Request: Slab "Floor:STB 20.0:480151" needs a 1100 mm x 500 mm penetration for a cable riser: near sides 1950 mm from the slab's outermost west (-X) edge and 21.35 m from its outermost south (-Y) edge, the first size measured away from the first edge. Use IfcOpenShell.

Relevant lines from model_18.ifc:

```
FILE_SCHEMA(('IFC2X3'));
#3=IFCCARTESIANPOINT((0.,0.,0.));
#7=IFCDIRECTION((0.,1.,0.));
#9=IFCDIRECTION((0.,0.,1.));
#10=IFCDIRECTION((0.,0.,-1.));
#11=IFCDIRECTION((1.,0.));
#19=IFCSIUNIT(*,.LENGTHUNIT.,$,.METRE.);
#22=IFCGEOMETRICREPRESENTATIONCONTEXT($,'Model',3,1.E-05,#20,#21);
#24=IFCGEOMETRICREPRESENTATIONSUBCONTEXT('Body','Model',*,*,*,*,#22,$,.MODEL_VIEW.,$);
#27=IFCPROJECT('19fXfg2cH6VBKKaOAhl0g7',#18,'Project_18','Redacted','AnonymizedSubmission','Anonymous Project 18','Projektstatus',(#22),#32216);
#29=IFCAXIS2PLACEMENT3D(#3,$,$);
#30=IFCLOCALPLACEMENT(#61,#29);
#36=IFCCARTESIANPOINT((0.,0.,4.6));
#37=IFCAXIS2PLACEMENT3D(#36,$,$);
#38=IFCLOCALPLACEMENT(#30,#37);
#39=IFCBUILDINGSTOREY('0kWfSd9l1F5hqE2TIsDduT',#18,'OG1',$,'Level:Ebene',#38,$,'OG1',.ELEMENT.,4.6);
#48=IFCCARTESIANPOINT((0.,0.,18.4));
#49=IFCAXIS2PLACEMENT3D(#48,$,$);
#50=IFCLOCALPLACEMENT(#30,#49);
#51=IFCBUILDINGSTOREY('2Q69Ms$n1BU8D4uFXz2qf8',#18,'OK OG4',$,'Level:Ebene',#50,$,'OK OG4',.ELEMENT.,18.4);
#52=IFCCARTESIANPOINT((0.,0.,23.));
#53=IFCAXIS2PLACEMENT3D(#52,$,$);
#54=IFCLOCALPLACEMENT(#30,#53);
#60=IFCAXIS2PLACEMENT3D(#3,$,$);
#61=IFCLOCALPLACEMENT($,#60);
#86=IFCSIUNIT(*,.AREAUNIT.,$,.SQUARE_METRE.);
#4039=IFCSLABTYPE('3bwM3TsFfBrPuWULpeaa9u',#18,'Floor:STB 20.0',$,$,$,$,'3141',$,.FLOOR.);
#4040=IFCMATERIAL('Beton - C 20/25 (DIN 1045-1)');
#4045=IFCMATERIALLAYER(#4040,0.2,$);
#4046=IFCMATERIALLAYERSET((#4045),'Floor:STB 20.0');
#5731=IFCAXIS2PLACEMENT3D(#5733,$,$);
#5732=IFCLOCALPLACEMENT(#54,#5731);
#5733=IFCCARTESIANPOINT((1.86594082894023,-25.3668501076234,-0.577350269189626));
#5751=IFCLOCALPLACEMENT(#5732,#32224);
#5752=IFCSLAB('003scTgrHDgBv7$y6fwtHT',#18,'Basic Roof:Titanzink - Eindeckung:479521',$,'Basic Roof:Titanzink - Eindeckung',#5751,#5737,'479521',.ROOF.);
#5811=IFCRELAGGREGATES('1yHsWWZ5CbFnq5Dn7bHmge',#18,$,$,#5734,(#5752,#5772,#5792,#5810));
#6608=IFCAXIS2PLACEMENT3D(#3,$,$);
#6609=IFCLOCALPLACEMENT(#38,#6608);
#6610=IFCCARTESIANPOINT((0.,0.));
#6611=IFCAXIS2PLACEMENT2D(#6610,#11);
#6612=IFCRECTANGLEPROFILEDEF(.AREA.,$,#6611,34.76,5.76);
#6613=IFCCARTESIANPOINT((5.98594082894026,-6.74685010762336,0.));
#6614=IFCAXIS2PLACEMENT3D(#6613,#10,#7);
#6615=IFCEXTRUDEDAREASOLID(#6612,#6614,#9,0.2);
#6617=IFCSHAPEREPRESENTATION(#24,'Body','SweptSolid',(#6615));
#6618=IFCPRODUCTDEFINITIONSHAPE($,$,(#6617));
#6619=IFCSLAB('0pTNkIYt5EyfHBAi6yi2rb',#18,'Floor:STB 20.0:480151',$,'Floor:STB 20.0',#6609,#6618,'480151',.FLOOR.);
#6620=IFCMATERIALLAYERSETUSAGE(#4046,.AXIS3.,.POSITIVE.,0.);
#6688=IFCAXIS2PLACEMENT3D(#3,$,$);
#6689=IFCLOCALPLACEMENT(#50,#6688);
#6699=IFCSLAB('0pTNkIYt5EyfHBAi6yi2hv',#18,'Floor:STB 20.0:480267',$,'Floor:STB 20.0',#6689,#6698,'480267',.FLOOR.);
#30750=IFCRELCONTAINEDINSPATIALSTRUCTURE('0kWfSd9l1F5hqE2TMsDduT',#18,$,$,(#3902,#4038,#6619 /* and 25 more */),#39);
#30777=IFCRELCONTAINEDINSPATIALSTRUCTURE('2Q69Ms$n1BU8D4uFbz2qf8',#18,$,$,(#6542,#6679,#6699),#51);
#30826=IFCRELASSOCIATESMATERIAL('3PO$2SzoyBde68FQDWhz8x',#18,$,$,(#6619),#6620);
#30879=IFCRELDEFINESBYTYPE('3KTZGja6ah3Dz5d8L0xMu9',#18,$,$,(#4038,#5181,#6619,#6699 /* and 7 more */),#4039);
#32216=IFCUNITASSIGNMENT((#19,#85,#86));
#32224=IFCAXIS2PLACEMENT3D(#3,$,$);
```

```python
import numpy as np
import ifcopenshell
import ifcopenshell.api.feature
import ifcopenshell.api.geometry
import ifcopenshell.api.root
import ifcopenshell.geom
import ifcopenshell.util.placement
import ifcopenshell.util.representation
import ifcopenshell.util.shape
import ifcopenshell.util.unit

model = ifcopenshell.open("model_18.ifc")
unit_scale = ifcopenshell.util.unit.calculate_unit_scale(model)
settings = ifcopenshell.geom.settings()


def volume(element):
    """Net volume in cubic metres, openings subtracted."""
    shape = ifcopenshell.geom.create_shape(settings, element)
    return ifcopenshell.util.shape.get_volume(shape.geometry)


slab = model.by_guid("0pTNkIYt5EyfHBAi6yi2rb")
before = volume(slab)

# Extent in the slab's own axes, in metres. The edges named are its -X and -Y sides.
slab_shape = ifcopenshell.geom.create_shape(settings, slab)
vertices = ifcopenshell.util.shape.get_vertices(slab_shape.geometry)
x_min, y_min, bottom = vertices.min(axis=0)
top = vertices[:, 2].max()

opening = ifcopenshell.api.root.create_entity(model, ifc_class="IfcOpeningElement", name="Cable riser opening")
context = ifcopenshell.util.representation.get_context(model, "Model", "Body", "MODEL_VIEW")
width, depth = 1.1, 0.5
outline = [(0.0, 0.0), (width, 0.0), (width, depth), (0.0, depth), (0.0, 0.0)]
# Overshoot both faces by 50 mm so the cut is clean.
shape = ifcopenshell.api.geometry.add_slab_representation(
    model, context=context, depth=top - bottom + 0.1, polyline=outline
)
ifcopenshell.api.geometry.assign_representation(model, product=opening, representation=shape)

matrix = ifcopenshell.util.placement.get_local_placement(slab.ObjectPlacement)
matrix[:, 3] = matrix @ np.append(np.array([x_min + 1.95, y_min + 21.35, bottom - 0.05]) / unit_scale, 1.0)
ifcopenshell.api.geometry.edit_object_placement(model, product=opening, matrix=matrix, is_si=False)
ifcopenshell.api.feature.add_feature(model, feature=opening, element=slab)

after = volume(slab)

print(f"slab volume {before:.3f} -> {after:.3f} m3")

model.write("model_18_updated.ifc")
```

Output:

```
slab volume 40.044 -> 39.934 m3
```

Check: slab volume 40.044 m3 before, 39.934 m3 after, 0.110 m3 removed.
